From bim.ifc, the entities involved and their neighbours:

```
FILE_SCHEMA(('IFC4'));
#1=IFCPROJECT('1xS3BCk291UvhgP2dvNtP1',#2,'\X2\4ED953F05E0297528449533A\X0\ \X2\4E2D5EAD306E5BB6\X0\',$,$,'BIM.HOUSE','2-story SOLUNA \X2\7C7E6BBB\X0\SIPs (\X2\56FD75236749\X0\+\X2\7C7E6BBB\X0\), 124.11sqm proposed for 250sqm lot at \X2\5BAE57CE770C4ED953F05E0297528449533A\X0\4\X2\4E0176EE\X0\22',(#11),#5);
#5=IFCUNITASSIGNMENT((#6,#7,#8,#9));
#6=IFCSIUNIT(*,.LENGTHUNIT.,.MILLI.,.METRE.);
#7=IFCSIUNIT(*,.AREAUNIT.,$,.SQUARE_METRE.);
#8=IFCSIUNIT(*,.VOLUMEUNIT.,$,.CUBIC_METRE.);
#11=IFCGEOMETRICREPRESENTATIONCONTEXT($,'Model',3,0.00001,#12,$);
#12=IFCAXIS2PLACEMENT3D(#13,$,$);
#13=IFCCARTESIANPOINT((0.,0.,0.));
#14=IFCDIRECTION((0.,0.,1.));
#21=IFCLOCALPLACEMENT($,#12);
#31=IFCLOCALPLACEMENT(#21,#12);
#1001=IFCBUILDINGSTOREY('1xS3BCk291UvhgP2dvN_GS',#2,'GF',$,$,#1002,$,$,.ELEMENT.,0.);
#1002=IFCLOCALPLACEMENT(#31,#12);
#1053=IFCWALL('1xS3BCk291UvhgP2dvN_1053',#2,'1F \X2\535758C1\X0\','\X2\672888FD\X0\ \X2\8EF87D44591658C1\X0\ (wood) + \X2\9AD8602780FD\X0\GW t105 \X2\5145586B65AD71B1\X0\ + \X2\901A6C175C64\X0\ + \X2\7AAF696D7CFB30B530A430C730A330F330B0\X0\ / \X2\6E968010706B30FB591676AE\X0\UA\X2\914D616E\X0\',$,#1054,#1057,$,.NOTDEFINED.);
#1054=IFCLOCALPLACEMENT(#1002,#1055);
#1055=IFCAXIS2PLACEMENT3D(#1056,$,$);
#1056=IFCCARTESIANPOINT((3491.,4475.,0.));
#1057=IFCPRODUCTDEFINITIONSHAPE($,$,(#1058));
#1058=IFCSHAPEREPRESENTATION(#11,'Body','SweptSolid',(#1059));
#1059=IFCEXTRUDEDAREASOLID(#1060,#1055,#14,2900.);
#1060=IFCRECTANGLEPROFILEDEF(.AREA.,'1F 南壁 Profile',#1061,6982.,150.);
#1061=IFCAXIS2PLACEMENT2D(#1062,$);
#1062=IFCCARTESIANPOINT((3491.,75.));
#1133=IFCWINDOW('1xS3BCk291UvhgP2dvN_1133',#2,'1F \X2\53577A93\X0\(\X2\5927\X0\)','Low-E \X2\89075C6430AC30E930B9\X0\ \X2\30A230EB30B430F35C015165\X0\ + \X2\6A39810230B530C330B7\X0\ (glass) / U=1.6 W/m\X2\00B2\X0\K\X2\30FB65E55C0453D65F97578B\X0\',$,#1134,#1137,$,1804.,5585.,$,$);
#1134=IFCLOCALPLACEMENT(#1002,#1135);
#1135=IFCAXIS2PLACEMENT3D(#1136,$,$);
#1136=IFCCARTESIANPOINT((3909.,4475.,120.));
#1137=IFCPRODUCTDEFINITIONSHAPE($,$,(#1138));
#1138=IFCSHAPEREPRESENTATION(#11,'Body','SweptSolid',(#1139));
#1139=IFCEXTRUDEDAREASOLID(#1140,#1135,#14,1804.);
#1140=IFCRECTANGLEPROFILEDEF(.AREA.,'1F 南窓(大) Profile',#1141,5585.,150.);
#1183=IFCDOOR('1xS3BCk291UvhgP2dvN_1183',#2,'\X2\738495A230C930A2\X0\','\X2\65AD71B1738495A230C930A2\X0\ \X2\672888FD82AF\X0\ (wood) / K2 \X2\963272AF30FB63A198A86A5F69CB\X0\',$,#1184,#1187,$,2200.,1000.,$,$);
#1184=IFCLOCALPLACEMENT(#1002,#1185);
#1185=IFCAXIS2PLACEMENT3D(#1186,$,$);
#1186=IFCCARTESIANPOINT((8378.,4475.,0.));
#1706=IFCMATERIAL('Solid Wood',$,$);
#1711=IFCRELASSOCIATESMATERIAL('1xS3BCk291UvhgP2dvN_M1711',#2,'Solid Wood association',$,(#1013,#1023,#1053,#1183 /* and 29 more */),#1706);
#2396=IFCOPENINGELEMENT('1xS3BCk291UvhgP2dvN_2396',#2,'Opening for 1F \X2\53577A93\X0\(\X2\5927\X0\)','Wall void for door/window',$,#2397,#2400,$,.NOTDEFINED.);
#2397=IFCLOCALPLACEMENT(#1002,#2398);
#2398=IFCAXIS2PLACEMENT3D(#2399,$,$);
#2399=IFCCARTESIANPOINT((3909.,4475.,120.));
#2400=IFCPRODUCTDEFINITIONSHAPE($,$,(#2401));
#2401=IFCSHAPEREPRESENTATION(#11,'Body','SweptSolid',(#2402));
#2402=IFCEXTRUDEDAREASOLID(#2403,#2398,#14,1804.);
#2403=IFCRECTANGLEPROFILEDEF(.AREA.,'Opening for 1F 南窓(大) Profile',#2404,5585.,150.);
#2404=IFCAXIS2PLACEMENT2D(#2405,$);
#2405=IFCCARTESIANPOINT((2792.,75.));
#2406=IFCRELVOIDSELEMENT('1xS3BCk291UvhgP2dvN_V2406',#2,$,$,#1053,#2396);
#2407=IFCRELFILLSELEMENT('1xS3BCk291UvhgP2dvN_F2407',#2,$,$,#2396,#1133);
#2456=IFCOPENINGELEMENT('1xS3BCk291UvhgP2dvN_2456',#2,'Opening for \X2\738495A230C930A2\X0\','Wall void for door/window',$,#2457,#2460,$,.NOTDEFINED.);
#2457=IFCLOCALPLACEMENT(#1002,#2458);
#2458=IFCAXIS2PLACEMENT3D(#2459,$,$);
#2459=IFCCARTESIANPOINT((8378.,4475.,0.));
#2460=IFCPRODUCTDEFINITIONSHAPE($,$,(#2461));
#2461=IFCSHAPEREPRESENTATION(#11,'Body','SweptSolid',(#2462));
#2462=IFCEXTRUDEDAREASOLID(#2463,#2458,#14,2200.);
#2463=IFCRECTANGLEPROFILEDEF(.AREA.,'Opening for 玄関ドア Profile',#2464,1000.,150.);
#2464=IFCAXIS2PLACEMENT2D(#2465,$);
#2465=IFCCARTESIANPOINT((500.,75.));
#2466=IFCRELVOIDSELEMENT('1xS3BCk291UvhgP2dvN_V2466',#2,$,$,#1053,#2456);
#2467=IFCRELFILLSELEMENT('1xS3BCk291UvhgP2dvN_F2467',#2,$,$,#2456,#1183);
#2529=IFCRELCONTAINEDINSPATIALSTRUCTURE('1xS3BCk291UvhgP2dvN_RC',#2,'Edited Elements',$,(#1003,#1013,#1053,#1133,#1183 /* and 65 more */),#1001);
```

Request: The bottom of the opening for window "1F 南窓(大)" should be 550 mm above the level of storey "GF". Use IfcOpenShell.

```python
import numpy as np
import ifcopenshell
import ifcopenshell.api.geometry
import ifcopenshell.geom
import ifcopenshell.util.element
import ifcopenshell.util.placement
import ifcopenshell.util.shape
import ifcopenshell.util.unit

model = ifcopenshell.open("bim.ifc")
unit_scale = ifcopenshell.util.unit.calculate_unit_scale(model)

window = model.by_guid("1xS3BCk291UvhgP2dvN_1133")
opening = window.FillsVoids[0].RelatingOpeningElement
storey = ifcopenshell.util.element.get_container(window, ifc_class="IfcBuildingStorey")
level = ifcopenshell.util.placement.get_local_placement(storey.ObjectPlacement)[2, 3]

# The opening's origin need not be at the sill, so measure its lowest point.
shape = ifcopenshell.geom.create_shape(ifcopenshell.geom.settings(), opening)
bottom = ifcopenshell.util.shape.get_shape_bottom_elevation(shape, shape.geometry) / unit_scale
dz = level + 550.0 - bottom

shift = np.array([0.0, 0.0, dz])
# The window is not placed relative to its opening, so move both.
for product in (opening, window):
    matrix = ifcopenshell.util.placement.get_local_placement(product.ObjectPlacement)
    matrix[:3, 3] += shift
    ifcopenshell.api.geometry.edit_object_placement(model, product=product, matrix=matrix, is_si=False)

print(f"moved by {dz * unit_scale:+.3f} m")

model.write("bim_edited.ifc")
```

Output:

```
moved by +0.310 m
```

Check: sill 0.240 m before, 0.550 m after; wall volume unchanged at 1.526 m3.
